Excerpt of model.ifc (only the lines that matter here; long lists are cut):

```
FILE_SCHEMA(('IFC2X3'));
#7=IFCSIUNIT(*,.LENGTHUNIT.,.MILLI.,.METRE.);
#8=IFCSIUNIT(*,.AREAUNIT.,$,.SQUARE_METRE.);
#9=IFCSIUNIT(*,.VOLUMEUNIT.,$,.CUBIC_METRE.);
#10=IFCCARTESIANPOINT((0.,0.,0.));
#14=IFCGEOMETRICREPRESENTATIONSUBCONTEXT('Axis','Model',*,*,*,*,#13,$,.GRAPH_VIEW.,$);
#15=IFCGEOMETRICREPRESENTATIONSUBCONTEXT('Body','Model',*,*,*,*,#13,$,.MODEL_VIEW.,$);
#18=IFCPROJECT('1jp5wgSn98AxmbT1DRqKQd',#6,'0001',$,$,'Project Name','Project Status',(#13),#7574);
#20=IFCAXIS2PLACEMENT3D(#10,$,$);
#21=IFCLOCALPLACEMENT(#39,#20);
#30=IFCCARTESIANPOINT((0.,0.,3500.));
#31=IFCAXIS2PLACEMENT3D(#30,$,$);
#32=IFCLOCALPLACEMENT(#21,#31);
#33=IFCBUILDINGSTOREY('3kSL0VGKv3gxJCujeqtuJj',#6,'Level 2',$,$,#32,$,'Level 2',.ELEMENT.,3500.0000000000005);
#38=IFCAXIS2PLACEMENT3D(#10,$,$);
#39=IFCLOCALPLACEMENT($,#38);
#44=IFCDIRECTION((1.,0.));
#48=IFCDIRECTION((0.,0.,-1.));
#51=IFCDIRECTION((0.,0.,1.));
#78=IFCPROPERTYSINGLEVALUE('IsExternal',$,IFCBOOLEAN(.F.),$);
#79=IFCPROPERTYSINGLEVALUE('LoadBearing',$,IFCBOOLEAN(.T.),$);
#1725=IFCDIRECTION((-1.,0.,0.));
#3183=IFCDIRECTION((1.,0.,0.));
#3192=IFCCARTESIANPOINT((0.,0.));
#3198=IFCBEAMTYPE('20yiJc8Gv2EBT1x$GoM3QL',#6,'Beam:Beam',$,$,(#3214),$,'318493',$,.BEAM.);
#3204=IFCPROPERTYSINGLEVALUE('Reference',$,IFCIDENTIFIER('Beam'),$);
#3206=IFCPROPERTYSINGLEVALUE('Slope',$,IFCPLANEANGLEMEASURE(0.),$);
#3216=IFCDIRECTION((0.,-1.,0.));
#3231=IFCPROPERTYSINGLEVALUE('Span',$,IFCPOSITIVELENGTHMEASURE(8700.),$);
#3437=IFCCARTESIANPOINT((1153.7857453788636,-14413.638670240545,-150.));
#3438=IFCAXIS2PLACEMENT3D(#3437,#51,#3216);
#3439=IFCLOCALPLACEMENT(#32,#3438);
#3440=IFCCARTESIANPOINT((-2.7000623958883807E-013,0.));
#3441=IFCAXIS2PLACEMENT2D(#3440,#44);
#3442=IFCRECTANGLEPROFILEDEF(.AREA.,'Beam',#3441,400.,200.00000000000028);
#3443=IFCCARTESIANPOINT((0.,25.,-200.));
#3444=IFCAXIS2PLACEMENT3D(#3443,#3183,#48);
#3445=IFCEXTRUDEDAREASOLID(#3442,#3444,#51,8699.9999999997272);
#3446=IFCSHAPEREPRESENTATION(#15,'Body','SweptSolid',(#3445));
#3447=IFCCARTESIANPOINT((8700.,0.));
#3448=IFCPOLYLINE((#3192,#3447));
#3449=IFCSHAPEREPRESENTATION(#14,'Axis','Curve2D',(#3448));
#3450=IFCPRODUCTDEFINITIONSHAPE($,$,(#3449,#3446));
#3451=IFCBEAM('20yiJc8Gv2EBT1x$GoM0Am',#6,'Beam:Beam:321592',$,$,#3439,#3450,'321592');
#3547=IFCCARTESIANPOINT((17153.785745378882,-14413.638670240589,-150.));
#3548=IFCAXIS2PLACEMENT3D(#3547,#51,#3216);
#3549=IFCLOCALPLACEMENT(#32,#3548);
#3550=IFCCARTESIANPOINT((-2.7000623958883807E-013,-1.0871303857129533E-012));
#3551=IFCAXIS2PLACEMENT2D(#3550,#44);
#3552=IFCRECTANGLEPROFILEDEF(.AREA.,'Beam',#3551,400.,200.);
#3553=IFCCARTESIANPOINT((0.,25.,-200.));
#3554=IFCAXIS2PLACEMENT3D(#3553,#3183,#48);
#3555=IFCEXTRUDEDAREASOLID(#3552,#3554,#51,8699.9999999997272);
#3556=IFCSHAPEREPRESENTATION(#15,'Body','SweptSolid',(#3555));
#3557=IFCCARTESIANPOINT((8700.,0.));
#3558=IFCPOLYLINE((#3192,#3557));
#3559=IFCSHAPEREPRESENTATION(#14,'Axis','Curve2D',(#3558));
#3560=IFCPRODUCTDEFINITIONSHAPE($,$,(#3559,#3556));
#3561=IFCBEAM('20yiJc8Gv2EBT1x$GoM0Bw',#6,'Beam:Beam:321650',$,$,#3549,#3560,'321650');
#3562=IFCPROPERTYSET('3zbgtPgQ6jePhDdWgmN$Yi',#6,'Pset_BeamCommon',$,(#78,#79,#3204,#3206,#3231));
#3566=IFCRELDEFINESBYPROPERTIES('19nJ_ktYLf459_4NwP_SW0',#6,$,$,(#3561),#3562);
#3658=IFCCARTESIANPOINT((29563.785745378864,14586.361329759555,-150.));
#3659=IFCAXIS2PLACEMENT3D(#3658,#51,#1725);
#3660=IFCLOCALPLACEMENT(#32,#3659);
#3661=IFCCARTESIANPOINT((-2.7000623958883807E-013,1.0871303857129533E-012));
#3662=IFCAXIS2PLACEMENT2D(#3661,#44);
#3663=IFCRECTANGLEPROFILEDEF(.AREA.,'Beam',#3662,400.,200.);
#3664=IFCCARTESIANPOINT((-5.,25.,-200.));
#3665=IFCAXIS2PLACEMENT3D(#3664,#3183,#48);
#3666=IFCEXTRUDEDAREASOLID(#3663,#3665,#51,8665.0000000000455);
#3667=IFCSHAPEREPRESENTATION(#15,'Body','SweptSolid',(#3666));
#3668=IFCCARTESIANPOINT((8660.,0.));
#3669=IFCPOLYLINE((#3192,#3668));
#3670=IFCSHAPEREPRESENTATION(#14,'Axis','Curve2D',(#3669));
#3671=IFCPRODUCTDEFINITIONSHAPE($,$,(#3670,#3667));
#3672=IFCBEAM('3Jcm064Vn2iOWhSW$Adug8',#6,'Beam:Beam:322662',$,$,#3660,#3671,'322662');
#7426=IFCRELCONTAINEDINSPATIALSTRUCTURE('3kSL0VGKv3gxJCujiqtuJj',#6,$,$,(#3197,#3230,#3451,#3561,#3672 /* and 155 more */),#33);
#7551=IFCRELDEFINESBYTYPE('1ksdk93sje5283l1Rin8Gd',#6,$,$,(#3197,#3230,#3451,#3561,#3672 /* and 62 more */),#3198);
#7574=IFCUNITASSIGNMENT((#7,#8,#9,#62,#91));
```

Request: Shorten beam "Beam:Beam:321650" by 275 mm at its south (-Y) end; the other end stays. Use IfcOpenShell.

```python
import numpy as np
import ifcopenshell
import ifcopenshell.api.pset
import ifcopenshell.util.element
import ifcopenshell.util.representation
import ifcopenshell.util.unit

model = ifcopenshell.open("model.ifc")
unit_scale = ifcopenshell.util.unit.calculate_unit_scale(model)

member = model.by_guid("20yiJc8Gv2EBT1x$GoM0Bw")
change = -0.275 / unit_scale

# The extrusion runs towards the end named, so only its depth changes.
body = ifcopenshell.util.representation.get_representation(member, "Model", "Body")
solid = body.Items[0]
old_length = solid.Depth
solid.Depth += change

# Move the axis end point with it.
axis = next(r for r in member.Representation.Representations if r.RepresentationIdentifier == "Axis").Items[0]
start, end = (np.array(p.Coordinates) for p in axis.Points)
end = end + (end - start) / np.linalg.norm(end - start) * change
point = model.createIfcCartesianPoint(end.tolist())
axis.Points = [axis.Points[0], point]

# Update the stored length and volume.
pset = model.by_id(ifcopenshell.util.element.get_pset(member, "Pset_BeamCommon", should_inherit=False)["id"])
ifcopenshell.api.pset.edit_pset(model, pset=pset, properties={
    "Span": model.create_entity("IfcPositiveLengthMeasure", solid.Depth),
})

print(f"length {old_length:g} -> {solid.Depth:g}")

model.write("model_updated.ifc")
```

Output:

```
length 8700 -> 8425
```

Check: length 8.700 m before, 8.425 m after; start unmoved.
